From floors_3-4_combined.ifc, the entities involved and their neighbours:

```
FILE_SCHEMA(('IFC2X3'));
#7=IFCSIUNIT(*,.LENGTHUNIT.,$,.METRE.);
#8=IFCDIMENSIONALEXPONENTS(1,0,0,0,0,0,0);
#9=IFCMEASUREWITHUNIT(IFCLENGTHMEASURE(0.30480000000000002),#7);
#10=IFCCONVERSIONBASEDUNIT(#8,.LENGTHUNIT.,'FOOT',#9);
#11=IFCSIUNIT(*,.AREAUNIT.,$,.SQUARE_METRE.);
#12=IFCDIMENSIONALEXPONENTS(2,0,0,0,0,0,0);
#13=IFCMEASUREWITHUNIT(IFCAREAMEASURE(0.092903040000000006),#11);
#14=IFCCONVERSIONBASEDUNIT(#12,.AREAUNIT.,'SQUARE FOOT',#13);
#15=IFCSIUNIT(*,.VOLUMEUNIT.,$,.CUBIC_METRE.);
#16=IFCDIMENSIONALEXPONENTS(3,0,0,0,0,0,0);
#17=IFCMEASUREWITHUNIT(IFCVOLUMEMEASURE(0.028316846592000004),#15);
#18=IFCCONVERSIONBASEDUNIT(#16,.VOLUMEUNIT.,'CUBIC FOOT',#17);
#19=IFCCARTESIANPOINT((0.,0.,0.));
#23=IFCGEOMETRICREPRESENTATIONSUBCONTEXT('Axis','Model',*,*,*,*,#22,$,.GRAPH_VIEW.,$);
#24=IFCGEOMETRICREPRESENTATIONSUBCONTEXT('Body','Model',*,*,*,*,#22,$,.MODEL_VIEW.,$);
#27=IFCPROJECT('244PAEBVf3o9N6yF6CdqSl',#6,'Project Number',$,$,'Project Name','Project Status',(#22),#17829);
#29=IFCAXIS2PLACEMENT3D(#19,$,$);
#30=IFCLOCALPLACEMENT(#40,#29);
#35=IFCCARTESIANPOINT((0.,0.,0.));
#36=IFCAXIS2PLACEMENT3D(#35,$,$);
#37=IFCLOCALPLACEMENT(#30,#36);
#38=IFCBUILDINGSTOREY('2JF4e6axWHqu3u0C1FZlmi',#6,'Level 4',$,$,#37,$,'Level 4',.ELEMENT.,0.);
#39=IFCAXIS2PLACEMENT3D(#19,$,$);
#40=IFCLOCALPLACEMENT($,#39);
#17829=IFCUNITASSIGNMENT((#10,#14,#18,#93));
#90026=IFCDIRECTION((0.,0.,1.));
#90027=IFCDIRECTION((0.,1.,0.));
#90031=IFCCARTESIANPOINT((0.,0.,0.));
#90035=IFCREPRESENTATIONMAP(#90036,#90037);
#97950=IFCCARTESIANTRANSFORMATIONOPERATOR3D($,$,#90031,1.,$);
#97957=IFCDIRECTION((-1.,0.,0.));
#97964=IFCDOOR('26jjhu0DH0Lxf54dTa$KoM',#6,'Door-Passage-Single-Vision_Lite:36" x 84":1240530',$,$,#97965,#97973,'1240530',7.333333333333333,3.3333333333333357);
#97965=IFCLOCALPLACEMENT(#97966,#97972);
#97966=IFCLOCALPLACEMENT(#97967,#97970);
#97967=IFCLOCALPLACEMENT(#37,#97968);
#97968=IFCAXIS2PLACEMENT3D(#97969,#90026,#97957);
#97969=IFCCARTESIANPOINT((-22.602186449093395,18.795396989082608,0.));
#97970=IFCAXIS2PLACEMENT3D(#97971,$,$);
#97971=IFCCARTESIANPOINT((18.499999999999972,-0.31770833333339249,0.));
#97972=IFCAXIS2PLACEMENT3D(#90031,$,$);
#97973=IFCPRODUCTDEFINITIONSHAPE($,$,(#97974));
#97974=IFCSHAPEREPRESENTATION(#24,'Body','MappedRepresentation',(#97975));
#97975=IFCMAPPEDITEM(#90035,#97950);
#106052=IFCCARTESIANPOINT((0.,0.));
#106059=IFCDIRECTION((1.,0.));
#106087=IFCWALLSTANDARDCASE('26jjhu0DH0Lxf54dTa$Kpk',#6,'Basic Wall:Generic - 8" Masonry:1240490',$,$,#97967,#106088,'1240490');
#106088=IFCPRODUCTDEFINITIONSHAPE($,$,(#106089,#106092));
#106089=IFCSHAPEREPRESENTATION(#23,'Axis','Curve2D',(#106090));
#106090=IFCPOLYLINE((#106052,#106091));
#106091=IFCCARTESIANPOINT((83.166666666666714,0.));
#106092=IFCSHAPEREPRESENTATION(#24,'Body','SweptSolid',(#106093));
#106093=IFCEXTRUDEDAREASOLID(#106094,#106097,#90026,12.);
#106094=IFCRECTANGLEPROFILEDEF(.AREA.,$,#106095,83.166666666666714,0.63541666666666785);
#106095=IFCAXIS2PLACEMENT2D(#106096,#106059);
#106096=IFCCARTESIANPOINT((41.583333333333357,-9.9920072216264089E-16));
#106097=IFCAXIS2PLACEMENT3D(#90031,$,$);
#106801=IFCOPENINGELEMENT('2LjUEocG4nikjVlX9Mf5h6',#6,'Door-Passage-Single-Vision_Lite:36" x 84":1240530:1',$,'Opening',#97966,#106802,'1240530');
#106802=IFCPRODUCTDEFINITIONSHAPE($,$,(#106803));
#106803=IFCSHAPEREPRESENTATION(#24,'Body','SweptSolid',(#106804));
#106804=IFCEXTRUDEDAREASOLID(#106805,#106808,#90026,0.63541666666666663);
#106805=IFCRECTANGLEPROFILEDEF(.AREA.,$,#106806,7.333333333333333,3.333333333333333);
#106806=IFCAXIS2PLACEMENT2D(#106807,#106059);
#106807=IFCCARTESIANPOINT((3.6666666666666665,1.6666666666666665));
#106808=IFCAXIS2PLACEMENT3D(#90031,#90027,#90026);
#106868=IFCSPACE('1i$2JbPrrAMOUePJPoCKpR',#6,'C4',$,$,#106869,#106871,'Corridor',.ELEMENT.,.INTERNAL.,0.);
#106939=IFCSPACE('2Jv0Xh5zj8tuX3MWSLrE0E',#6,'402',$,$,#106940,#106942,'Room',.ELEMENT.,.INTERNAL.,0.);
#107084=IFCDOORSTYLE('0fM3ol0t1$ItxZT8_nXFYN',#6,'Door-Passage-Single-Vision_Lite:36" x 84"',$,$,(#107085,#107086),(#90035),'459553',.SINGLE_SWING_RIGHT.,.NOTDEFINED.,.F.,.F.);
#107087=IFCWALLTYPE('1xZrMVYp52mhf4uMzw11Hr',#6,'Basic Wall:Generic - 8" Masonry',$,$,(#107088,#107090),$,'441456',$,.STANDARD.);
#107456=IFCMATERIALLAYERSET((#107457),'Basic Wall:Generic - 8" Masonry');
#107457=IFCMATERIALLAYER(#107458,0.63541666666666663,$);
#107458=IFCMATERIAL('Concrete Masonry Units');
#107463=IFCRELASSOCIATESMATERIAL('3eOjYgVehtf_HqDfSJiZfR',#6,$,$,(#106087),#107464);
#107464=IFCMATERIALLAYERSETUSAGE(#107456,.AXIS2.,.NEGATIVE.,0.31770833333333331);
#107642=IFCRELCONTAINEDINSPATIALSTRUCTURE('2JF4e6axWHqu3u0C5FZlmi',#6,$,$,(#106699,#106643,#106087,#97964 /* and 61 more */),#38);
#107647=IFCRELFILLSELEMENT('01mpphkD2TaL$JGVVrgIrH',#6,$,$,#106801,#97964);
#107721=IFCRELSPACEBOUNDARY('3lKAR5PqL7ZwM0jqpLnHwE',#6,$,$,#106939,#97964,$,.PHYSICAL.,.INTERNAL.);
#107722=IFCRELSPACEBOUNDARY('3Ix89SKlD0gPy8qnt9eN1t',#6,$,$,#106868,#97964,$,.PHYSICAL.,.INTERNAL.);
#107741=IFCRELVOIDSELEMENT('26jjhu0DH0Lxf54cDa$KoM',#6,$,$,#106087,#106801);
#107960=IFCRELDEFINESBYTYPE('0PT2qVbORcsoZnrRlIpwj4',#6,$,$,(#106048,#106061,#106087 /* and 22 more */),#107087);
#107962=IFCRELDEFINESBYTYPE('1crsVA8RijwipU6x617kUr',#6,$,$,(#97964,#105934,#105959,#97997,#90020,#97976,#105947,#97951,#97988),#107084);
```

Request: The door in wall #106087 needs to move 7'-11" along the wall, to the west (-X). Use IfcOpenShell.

```python
import ifcopenshell
import ifcopenshell.api.geometry
import ifcopenshell.util.placement
import ifcopenshell.util.unit

model = ifcopenshell.open("floors_3-4_combined.ifc")
unit_scale = ifcopenshell.util.unit.calculate_unit_scale(model)

door = model.by_id(97964)
opening = door.FillsVoids[0].RelatingOpeningElement
wall = opening.VoidsElements[0].RelatingBuildingElement

wall_matrix = ifcopenshell.util.placement.get_local_placement(wall.ObjectPlacement)
shift = wall_matrix[:3, 0] * 95 * 0.0254 / unit_scale
before = ifcopenshell.util.placement.get_local_placement(door.ObjectPlacement)[:3, 3].copy()

# The door is placed relative to its opening, so it follows when the opening moves.
matrix = ifcopenshell.util.placement.get_local_placement(opening.ObjectPlacement)
matrix[:3, 3] += shift
ifcopenshell.api.geometry.edit_object_placement(
    model, product=opening, matrix=matrix, is_si=False, should_transform_children=True
)

after = ifcopenshell.util.placement.get_local_placement(door.ObjectPlacement)[:3, 3]
print("door moved by", (after - before).round(3) + 0.0)

model.write("floors_3-4_combined-out.ifc")
```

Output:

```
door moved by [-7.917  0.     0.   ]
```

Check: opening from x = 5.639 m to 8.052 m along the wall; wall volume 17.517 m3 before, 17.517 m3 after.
